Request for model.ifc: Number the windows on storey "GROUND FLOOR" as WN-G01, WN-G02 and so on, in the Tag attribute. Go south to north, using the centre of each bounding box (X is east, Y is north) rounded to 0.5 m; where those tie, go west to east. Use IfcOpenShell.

First a look at what the model holds.

```python
import ifcopenshell
import ifcopenshell.util.element
import ifcopenshell.util.placement

model = ifcopenshell.open("model.ifc")
print(model.schema)
storey = next(s for s in model.by_type("IfcBuildingStorey") if s.Name == "GROUND FLOOR")
windows = [e for e in ifcopenshell.util.element.get_decomposition(storey) if e.is_a("IfcWindow")]
for e in sorted(windows, key=lambda e: e.id()):
    origin = ifcopenshell.util.placement.get_local_placement(e.ObjectPlacement)[:3, 3]
    print(e.id(), e.Tag, e.Name, origin.round(2) + 0.0, sep=" | ")
```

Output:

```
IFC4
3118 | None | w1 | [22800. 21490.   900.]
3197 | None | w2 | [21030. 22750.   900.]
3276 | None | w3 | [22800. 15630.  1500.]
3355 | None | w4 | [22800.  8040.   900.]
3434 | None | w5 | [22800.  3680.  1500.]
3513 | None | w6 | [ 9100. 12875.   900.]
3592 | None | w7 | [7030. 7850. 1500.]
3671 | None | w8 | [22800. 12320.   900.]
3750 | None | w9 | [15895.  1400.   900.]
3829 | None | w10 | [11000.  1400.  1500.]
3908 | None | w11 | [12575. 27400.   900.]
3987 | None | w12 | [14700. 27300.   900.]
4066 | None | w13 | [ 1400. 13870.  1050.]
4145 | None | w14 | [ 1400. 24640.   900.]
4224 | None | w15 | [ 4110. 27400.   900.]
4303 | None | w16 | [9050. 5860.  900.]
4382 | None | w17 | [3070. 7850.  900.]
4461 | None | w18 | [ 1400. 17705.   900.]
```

```python
import ifcopenshell
import ifcopenshell.geom
import ifcopenshell.util.element
import ifcopenshell.util.shape

model = ifcopenshell.open("model.ifc")
settings = ifcopenshell.geom.settings()
settings.set("use-world-coords", True)


def centre(element):
    shape = ifcopenshell.geom.create_shape(settings, element)
    return ifcopenshell.util.shape.get_bbox_centroid(shape.geometry)


storey = next(s for s in model.by_type("IfcBuildingStorey") if s.Name == "GROUND FLOOR")
windows = [e for e in ifcopenshell.util.element.get_decomposition(storey) if e.is_a("IfcWindow")]

# Insertion points can sit at a corner or the storey origin, so sort by the geometry (in metres).
centres = {e: centre(e) for e in windows}
windows.sort(key=lambda e: (round(centres[e][1] / 0.5), centres[e][0]))

for i, e in enumerate(windows, start=1):
    number = f"WN-G{i:02d}"
    e.Tag = number
    print(e.id(), number)

model.write("model_edited.ifc")
```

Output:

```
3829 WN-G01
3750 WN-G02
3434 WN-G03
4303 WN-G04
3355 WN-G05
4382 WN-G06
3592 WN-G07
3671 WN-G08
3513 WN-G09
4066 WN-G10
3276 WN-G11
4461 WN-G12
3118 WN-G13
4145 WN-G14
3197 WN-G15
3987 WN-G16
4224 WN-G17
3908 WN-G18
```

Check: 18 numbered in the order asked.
